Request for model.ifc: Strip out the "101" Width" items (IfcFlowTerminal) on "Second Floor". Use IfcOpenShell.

First a look at what the model holds.

```python
import ifcopenshell
import ifcopenshell.util.element

model = ifcopenshell.open("model.ifc")
print(model.schema)
storey = next(s for s in model.by_type("IfcBuildingStorey") if s.Name == "Second Floor")
terminals = [e for e in ifcopenshell.util.element.get_decomposition(storey) if e.is_a("IfcFlowTerminal")]
seen = {}
for e in terminals:
    element_type = ifcopenshell.util.element.get_type(e)
    name = element_type.Name if element_type not in (None, e) else None
    seen[name] = seen.get(name, 0) + 1
for name, count in sorted(seen.items(), key=str):
    print(count, "x", name)
```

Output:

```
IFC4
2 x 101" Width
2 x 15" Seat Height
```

```python
import ifcopenshell
import ifcopenshell.api.root
import ifcopenshell.util.element

model = ifcopenshell.open("model.ifc")

storey = next(s for s in model.by_type("IfcBuildingStorey") if s.Name == "Second Floor")
terminals = [e for e in ifcopenshell.util.element.get_decomposition(storey) if e.is_a("IfcFlowTerminal")]
targets = [e for e in terminals if (t := ifcopenshell.util.element.get_type(e)) not in (None, e) and t.Name == '101" Width']

for e in targets:
    ifcopenshell.api.root.remove_product(model, product=e)
print(len(targets), "removed")

model.write("model_rev.ifc")
```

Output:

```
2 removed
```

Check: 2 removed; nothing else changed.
